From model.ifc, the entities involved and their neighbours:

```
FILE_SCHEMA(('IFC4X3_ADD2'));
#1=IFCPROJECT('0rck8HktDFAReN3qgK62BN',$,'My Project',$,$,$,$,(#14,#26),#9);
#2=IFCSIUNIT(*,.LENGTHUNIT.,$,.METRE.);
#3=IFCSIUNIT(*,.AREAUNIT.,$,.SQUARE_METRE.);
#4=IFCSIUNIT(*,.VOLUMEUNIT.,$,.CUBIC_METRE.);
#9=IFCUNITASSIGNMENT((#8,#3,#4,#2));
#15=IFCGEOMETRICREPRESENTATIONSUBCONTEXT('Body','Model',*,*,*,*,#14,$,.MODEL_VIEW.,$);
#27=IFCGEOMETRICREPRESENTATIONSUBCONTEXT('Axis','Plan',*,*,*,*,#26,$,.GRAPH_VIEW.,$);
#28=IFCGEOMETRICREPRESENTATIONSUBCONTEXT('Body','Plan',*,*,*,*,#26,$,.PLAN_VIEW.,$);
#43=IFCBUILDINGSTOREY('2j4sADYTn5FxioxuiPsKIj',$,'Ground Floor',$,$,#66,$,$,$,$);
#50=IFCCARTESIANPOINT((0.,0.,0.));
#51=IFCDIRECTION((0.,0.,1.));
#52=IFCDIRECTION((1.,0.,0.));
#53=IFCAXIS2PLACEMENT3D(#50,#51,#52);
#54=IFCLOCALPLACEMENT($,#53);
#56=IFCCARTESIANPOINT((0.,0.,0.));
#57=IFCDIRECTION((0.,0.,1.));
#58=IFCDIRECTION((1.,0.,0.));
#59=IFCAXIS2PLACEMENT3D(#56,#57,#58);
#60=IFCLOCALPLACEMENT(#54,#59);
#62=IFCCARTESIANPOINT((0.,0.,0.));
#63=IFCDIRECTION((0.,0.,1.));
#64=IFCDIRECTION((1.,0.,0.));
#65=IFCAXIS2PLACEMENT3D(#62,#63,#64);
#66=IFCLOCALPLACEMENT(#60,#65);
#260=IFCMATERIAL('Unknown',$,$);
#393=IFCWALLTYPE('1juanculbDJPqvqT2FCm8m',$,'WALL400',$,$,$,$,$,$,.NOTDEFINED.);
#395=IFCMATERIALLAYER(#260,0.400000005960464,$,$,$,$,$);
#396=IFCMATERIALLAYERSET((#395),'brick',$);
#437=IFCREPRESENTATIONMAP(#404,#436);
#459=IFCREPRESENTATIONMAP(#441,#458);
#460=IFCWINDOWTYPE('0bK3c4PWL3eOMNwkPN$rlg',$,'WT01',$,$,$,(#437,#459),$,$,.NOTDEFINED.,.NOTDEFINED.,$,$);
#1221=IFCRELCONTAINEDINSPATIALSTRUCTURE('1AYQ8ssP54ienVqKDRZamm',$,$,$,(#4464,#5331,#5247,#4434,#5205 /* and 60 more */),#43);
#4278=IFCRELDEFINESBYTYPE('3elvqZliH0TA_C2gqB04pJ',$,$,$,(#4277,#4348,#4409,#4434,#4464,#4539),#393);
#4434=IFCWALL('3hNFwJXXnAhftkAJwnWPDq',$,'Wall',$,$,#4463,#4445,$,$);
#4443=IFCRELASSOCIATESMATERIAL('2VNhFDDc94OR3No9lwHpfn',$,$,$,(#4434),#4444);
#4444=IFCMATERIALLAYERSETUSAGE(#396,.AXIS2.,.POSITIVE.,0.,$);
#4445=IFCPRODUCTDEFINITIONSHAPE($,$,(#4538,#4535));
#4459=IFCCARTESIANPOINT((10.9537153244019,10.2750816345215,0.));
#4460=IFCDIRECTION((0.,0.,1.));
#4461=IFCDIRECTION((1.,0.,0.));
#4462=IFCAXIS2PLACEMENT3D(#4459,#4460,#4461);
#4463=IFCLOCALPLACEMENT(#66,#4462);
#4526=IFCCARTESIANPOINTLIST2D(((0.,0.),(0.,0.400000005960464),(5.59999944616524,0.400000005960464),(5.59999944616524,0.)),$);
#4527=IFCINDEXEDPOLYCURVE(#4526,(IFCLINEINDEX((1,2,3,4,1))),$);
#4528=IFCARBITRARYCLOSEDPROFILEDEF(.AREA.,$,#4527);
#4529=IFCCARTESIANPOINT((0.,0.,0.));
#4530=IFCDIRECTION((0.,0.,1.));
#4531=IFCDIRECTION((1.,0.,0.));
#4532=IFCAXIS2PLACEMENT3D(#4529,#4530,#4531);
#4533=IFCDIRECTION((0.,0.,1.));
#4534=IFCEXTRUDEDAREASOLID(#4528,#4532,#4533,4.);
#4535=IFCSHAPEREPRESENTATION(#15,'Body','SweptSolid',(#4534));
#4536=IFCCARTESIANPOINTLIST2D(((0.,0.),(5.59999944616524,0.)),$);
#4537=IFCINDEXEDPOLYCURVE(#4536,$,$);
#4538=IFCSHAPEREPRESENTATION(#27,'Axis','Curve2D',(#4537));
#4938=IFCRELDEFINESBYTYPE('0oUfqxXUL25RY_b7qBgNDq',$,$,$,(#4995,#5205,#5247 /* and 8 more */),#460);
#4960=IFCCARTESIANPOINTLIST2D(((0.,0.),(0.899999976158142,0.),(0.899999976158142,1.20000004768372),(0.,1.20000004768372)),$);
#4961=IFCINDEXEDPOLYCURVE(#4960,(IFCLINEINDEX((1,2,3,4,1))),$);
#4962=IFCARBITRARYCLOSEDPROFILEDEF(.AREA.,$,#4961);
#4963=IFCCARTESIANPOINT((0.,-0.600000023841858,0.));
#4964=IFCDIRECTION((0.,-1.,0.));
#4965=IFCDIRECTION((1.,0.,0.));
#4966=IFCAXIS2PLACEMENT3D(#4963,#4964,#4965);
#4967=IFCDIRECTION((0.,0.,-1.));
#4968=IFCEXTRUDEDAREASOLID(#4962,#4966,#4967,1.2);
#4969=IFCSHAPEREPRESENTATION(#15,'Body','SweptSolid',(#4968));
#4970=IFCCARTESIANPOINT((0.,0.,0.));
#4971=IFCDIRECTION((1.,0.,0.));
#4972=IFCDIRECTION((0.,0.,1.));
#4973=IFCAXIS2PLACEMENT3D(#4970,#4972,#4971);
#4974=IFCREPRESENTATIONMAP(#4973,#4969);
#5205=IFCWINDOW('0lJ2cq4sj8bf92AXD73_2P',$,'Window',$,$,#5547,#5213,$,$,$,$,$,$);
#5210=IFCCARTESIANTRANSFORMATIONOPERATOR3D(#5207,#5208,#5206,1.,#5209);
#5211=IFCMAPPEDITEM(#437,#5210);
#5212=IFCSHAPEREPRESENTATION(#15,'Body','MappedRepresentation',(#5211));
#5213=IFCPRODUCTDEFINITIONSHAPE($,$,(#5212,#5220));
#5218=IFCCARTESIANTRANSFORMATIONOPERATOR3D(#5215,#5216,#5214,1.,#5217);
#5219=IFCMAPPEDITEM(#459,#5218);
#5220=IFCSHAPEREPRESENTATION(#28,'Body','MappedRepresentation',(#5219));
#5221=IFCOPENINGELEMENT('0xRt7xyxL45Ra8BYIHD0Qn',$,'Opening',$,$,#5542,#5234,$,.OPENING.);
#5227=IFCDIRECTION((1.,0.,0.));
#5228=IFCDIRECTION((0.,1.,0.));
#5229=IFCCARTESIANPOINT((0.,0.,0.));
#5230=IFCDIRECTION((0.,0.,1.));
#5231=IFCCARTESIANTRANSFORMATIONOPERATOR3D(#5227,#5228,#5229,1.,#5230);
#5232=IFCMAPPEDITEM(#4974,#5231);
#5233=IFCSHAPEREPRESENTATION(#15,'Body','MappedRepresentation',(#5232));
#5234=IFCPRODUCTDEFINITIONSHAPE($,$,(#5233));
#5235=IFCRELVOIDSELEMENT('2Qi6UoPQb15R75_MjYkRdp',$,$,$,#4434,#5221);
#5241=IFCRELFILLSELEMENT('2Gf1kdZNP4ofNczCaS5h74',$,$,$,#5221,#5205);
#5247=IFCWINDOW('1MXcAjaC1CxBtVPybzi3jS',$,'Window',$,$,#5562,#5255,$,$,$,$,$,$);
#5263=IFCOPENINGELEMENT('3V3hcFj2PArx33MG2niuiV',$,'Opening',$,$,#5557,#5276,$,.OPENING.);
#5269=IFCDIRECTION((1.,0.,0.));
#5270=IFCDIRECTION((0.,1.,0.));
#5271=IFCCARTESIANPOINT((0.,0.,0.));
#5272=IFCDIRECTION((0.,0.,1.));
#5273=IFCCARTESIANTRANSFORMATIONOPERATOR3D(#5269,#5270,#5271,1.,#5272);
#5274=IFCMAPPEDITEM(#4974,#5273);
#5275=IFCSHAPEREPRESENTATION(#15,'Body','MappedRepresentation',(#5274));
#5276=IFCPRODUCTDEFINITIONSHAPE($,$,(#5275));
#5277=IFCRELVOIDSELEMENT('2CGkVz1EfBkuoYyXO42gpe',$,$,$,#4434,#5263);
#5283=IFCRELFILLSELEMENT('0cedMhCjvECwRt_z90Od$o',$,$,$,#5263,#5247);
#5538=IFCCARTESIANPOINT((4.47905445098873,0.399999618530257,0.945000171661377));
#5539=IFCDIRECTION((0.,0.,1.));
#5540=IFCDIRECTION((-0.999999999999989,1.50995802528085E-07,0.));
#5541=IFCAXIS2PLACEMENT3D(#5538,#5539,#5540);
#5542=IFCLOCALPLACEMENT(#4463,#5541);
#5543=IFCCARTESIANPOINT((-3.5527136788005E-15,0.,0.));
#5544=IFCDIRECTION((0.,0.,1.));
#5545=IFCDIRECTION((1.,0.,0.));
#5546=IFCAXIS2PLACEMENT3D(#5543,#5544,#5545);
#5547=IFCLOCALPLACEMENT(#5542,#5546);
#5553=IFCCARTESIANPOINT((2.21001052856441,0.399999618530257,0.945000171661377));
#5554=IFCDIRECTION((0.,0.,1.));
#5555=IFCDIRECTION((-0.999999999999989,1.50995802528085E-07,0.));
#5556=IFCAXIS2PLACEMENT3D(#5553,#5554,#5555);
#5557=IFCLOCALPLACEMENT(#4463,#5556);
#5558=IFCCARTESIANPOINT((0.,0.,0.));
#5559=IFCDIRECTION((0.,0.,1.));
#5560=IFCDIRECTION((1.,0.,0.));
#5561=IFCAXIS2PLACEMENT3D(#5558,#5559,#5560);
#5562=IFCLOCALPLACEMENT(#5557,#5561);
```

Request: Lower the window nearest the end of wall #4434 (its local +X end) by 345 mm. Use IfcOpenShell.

```python
import numpy as np
import ifcopenshell
import ifcopenshell.api.geometry
import ifcopenshell.util.placement
import ifcopenshell.util.unit

model = ifcopenshell.open("model.ifc")
unit_scale = ifcopenshell.util.unit.calculate_unit_scale(model)

window = model.by_guid("0lJ2cq4sj8bf92AXD73_2P")
opening = window.FillsVoids[0].RelatingOpeningElement
dz = -0.345 / unit_scale

shift = np.array([0.0, 0.0, dz])
# The window is placed relative to its opening, so it follows when the opening moves.
matrix = ifcopenshell.util.placement.get_local_placement(opening.ObjectPlacement)
matrix[:3, 3] += shift
ifcopenshell.api.geometry.edit_object_placement(
    model, product=opening, matrix=matrix, is_si=False, should_transform_children=True
)

print(f"moved by {dz * unit_scale:+.3f} m")

model.write("model_edited.ifc")
```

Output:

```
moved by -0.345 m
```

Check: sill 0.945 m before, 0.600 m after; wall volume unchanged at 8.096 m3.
